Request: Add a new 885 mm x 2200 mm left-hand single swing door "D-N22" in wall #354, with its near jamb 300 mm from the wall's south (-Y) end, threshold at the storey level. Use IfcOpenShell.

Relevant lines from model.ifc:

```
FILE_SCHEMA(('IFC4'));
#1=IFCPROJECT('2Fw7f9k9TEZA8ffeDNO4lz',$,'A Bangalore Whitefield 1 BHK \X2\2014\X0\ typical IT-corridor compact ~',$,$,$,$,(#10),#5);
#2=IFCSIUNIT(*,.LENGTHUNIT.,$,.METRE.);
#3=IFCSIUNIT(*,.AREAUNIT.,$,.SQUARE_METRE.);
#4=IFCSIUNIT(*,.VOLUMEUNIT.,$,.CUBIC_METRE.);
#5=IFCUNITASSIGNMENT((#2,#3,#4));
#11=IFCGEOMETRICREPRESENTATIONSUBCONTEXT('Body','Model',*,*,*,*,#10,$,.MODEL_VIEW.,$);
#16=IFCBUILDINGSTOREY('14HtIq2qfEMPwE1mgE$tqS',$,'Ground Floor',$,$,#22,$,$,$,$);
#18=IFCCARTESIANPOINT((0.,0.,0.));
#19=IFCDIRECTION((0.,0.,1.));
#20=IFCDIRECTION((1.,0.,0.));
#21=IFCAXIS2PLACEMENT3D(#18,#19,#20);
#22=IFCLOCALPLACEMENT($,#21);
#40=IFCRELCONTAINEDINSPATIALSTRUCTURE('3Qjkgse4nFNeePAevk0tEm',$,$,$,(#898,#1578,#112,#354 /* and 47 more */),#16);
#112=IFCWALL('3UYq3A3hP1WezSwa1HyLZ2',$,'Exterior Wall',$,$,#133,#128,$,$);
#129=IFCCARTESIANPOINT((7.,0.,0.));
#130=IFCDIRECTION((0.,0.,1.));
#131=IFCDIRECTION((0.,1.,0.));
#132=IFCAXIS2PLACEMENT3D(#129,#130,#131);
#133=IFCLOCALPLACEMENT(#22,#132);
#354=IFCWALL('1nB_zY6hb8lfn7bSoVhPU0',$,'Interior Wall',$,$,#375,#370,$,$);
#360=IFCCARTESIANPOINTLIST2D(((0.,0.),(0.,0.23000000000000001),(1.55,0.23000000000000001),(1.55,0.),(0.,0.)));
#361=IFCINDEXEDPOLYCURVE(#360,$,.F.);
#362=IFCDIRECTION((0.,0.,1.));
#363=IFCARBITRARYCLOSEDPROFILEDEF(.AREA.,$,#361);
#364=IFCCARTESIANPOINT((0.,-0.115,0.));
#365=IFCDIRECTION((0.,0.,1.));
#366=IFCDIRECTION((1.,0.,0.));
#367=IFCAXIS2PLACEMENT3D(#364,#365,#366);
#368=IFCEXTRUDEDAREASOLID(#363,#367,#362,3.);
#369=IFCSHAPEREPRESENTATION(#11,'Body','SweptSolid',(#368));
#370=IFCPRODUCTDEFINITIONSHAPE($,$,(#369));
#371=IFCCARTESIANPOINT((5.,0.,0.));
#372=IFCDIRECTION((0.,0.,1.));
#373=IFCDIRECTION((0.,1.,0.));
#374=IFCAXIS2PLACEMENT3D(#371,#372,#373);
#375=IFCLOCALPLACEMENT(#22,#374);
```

```python
import numpy as np
import ifcopenshell
import ifcopenshell.api.feature
import ifcopenshell.api.geometry
import ifcopenshell.api.root
import ifcopenshell.api.spatial
import ifcopenshell.geom
import ifcopenshell.util.element
import ifcopenshell.util.placement
import ifcopenshell.util.representation
import ifcopenshell.util.shape
import ifcopenshell.util.unit

model = ifcopenshell.open("model.ifc")
unit_scale = ifcopenshell.util.unit.calculate_unit_scale(model)
settings = ifcopenshell.geom.settings()


def volume(element):
    """Net volume in cubic metres, openings subtracted."""
    shape = ifcopenshell.geom.create_shape(settings, element)
    return ifcopenshell.util.shape.get_volume(shape.geometry)


wall = model.by_guid("1nB_zY6hb8lfn7bSoVhPU0")
storey = ifcopenshell.util.element.get_container(wall, ifc_class="IfcBuildingStorey")
context = ifcopenshell.util.representation.get_context(model, "Model", "Body", "MODEL_VIEW")
before = volume(wall)

width, height, from_end, sill = 0.885, 2.2, 0.3, 0.0  # metres

# The wall runs along its own X axis, and the end named is its -X end.
wall_shape = ifcopenshell.geom.create_shape(settings, wall)
x, y, z = ifcopenshell.util.shape.get_vertices(wall_shape.geometry).T
start = x.min() + from_end
face, thickness = float(y.min()), float(y.max() - y.min())
wall_matrix = ifcopenshell.util.placement.get_local_placement(wall.ObjectPlacement)
level = ifcopenshell.util.placement.get_local_placement(storey.ObjectPlacement)[2, 3]


def in_wall(x, y):
    """Placement at x, y metres in the wall's axes, at sill height."""
    matrix = wall_matrix.copy()
    matrix[:, 3] = wall_matrix @ np.array([x / unit_scale, y / unit_scale, 0.0, 1.0])
    matrix[2, 3] = level + sill / unit_scale
    return matrix


# Opening: a box that overshoots both wall faces by 50 mm.
opening = ifcopenshell.api.root.create_entity(model, ifc_class="IfcOpeningElement", predefined_type="OPENING")
box = ifcopenshell.api.geometry.add_wall_representation(
    model, context=context, length=width, height=height, thickness=thickness + 0.1
)
ifcopenshell.api.geometry.assign_representation(model, product=opening, representation=box)
ifcopenshell.api.geometry.edit_object_placement(model, product=opening, matrix=in_wall(start, face - 0.05), is_si=False)
ifcopenshell.api.feature.add_feature(model, feature=opening, element=wall)

door = ifcopenshell.api.root.create_entity(model, ifc_class="IfcDoor", name="D-N22", predefined_type="DOOR")
door.OverallWidth, door.OverallHeight = width / unit_scale, height / unit_scale
door.OperationType = "SINGLE_SWING_LEFT"
body = ifcopenshell.api.geometry.add_door_representation(
    model,
    context=context,
    overall_width=door.OverallWidth,
    overall_height=door.OverallHeight,
    operation_type="SINGLE_SWING_LEFT",
    lining_properties={"LiningDepth": thickness / unit_scale, "ThresholdDepth": thickness / unit_scale},
)
ifcopenshell.api.geometry.assign_representation(model, product=door, representation=body)
ifcopenshell.api.spatial.assign_container(model, products=[door], relating_structure=storey)
ifcopenshell.api.feature.add_filling(model, opening=opening, element=door)

# The lining spans the wall, so the door starts at the wall face.
ifcopenshell.api.geometry.edit_object_placement(model, product=door, matrix=in_wall(start, face), is_si=False)

after = volume(wall)

print(f"wall volume {before:.3f} -> {after:.3f} m3")

model.write("model_edited.ifc")
```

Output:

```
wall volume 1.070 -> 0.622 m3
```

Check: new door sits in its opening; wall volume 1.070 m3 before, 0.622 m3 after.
